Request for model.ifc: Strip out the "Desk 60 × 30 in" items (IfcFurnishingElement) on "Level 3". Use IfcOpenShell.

First a look at what the model holds.

```python
import ifcopenshell
import ifcopenshell.util.element

model = ifcopenshell.open("model.ifc")
print(model.schema)
storey = next(s for s in model.by_type("IfcBuildingStorey") if s.Name == "Level 3")
furniture = [e for e in ifcopenshell.util.element.get_decomposition(storey) if e.is_a("IfcFurnishingElement")]
seen = {}
for e in furniture:
    element_type = ifcopenshell.util.element.get_type(e)
    name = element_type.Name if element_type not in (None, e) else None
    seen[name] = seen.get(name, 0) + 1
for name, count in sorted(seen.items(), key=str):
    print(count, "x", name)
```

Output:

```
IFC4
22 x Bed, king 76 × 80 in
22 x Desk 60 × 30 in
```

```python
import ifcopenshell
import ifcopenshell.api.root
import ifcopenshell.util.element

model = ifcopenshell.open("model.ifc")

storey = next(s for s in model.by_type("IfcBuildingStorey") if s.Name == "Level 3")
furniture = [e for e in ifcopenshell.util.element.get_decomposition(storey) if e.is_a("IfcFurnishingElement")]
targets = [e for e in furniture if (t := ifcopenshell.util.element.get_type(e)) not in (None, e) and t.Name == "Desk 60 × 30 in"]

for e in targets:
    ifcopenshell.api.root.remove_product(model, product=e)
print(len(targets), "removed")

model.write("model_rev.ifc")
```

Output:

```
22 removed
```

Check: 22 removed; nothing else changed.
